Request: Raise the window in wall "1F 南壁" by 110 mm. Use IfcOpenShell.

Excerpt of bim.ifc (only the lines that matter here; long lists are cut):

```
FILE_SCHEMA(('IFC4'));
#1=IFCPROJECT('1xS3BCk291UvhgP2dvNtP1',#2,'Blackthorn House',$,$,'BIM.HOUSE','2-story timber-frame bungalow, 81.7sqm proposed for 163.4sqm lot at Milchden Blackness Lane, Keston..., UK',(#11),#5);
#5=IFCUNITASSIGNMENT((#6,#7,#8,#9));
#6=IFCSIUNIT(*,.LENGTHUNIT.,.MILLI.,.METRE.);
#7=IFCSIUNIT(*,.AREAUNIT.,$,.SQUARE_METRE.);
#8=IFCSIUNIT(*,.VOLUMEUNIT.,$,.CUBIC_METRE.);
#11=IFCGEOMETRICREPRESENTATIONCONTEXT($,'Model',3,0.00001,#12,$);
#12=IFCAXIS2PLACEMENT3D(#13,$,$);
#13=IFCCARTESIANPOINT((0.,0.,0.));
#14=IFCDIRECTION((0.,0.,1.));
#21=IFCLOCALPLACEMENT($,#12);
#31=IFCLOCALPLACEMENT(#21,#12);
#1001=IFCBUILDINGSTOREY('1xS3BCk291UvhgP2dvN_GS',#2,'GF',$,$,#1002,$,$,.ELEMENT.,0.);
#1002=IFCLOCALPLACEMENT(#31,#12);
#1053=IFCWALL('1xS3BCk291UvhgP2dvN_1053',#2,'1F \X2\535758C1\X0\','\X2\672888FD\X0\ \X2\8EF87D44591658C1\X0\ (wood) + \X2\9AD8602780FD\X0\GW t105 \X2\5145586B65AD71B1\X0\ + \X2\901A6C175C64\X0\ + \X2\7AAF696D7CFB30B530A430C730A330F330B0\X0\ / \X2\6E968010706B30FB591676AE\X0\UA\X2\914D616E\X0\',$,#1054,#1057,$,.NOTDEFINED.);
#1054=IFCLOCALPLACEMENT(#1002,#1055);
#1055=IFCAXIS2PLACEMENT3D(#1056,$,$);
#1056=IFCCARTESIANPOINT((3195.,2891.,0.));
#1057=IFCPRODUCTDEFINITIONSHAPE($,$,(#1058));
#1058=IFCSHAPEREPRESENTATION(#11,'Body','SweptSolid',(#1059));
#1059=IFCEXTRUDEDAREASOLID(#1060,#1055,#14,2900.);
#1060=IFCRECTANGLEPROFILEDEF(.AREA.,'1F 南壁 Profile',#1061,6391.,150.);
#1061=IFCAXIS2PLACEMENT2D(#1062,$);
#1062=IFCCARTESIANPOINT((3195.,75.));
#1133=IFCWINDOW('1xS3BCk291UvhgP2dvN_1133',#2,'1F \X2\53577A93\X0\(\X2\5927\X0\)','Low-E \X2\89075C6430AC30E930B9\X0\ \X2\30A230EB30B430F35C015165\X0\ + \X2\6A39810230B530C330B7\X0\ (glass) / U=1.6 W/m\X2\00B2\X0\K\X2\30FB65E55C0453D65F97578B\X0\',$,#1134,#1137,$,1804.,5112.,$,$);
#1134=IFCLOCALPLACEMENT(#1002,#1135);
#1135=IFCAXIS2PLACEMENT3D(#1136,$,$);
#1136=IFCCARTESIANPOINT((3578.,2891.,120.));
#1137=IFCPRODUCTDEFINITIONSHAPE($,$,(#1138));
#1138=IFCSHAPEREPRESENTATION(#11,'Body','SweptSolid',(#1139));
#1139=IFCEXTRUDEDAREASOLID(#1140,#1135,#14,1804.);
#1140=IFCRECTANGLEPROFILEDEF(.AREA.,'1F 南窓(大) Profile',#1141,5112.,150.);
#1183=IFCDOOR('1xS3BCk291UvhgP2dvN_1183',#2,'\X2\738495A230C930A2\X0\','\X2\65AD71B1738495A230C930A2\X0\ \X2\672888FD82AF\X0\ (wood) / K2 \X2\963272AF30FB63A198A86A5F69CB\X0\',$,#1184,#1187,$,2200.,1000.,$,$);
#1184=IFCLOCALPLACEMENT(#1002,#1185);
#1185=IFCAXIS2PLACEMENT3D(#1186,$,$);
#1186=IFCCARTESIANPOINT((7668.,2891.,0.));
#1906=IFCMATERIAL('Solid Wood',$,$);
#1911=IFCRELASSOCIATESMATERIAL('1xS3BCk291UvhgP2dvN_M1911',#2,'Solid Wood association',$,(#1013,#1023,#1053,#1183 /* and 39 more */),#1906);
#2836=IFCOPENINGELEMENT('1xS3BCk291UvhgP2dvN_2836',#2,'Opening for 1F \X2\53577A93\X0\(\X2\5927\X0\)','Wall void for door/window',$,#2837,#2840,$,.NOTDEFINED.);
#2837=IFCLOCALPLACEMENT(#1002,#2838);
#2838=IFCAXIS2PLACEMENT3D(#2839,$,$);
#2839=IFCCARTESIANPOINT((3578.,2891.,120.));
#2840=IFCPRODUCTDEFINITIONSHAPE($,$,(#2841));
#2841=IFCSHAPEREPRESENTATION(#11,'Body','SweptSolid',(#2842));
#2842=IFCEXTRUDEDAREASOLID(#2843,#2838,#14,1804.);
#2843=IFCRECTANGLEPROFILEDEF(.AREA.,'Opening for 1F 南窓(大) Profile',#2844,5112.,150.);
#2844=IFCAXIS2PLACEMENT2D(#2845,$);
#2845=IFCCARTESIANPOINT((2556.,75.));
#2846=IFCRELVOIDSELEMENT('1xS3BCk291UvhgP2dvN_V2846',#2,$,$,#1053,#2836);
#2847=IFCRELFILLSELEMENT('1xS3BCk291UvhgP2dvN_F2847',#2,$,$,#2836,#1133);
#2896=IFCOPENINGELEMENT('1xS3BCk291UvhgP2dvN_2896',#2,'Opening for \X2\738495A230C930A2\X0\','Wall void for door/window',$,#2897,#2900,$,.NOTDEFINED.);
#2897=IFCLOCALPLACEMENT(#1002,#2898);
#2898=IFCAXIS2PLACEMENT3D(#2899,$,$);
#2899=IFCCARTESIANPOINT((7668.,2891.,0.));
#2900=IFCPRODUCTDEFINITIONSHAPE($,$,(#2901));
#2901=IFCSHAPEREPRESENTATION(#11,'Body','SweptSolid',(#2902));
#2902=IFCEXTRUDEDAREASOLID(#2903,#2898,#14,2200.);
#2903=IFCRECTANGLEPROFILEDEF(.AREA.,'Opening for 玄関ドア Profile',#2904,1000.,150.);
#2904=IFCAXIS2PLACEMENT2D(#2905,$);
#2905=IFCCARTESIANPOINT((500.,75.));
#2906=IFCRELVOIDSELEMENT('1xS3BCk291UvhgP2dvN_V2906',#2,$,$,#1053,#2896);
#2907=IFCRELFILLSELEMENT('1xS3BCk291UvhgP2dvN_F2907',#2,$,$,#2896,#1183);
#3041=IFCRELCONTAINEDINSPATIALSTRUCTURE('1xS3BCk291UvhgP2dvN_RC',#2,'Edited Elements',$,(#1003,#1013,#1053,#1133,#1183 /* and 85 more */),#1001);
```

```python
import numpy as np
import ifcopenshell
import ifcopenshell.api.geometry
import ifcopenshell.util.placement
import ifcopenshell.util.unit

model = ifcopenshell.open("bim.ifc")
unit_scale = ifcopenshell.util.unit.calculate_unit_scale(model)

window = model.by_id(1133)
opening = window.FillsVoids[0].RelatingOpeningElement
dz = 0.11 / unit_scale

shift = np.array([0.0, 0.0, dz])
# The window is not placed relative to its opening, so move both.
for product in (opening, window):
    matrix = ifcopenshell.util.placement.get_local_placement(product.ObjectPlacement)
    matrix[:3, 3] += shift
    ifcopenshell.api.geometry.edit_object_placement(model, product=product, matrix=matrix, is_si=False)

print(f"moved by {dz * unit_scale:+.3f} m")

model.write("bim_v2.ifc")
```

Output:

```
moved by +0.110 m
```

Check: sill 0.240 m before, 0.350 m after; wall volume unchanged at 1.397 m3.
